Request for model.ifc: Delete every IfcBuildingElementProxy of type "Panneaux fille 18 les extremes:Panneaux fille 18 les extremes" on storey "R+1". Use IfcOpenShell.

First a look at what the model holds.

```python
import ifcopenshell
import ifcopenshell.util.element

model = ifcopenshell.open("model.ifc")
print(model.schema)
storey = next(s for s in model.by_type("IfcBuildingStorey") if s.Name == "R+1")
proxies = [e for e in ifcopenshell.util.element.get_decomposition(storey) if e.is_a("IfcBuildingElementProxy")]
seen = {}
for e in proxies:
    element_type = ifcopenshell.util.element.get_type(e)
    name = element_type.Name if element_type not in (None, e) else None
    seen[name] = seen.get(name, 0) + 1
for name, count in sorted(seen.items(), key=str):
    print(count, "x", name)
```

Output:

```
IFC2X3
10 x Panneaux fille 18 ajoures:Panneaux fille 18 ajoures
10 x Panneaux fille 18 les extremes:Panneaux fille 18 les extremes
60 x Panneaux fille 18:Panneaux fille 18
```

```python
import ifcopenshell
import ifcopenshell.api.root
import ifcopenshell.util.element

model = ifcopenshell.open("model.ifc")

storey = next(s for s in model.by_type("IfcBuildingStorey") if s.Name == "R+1")
proxies = [e for e in ifcopenshell.util.element.get_decomposition(storey) if e.is_a("IfcBuildingElementProxy")]
targets = [e for e in proxies if (t := ifcopenshell.util.element.get_type(e)) not in (None, e) and t.Name == "Panneaux fille 18 les extremes:Panneaux fille 18 les extremes"]

for e in targets:
    ifcopenshell.api.root.remove_product(model, product=e)
print(len(targets), "removed")

model.write("model_edited.ifc")
```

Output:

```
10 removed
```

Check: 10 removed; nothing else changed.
